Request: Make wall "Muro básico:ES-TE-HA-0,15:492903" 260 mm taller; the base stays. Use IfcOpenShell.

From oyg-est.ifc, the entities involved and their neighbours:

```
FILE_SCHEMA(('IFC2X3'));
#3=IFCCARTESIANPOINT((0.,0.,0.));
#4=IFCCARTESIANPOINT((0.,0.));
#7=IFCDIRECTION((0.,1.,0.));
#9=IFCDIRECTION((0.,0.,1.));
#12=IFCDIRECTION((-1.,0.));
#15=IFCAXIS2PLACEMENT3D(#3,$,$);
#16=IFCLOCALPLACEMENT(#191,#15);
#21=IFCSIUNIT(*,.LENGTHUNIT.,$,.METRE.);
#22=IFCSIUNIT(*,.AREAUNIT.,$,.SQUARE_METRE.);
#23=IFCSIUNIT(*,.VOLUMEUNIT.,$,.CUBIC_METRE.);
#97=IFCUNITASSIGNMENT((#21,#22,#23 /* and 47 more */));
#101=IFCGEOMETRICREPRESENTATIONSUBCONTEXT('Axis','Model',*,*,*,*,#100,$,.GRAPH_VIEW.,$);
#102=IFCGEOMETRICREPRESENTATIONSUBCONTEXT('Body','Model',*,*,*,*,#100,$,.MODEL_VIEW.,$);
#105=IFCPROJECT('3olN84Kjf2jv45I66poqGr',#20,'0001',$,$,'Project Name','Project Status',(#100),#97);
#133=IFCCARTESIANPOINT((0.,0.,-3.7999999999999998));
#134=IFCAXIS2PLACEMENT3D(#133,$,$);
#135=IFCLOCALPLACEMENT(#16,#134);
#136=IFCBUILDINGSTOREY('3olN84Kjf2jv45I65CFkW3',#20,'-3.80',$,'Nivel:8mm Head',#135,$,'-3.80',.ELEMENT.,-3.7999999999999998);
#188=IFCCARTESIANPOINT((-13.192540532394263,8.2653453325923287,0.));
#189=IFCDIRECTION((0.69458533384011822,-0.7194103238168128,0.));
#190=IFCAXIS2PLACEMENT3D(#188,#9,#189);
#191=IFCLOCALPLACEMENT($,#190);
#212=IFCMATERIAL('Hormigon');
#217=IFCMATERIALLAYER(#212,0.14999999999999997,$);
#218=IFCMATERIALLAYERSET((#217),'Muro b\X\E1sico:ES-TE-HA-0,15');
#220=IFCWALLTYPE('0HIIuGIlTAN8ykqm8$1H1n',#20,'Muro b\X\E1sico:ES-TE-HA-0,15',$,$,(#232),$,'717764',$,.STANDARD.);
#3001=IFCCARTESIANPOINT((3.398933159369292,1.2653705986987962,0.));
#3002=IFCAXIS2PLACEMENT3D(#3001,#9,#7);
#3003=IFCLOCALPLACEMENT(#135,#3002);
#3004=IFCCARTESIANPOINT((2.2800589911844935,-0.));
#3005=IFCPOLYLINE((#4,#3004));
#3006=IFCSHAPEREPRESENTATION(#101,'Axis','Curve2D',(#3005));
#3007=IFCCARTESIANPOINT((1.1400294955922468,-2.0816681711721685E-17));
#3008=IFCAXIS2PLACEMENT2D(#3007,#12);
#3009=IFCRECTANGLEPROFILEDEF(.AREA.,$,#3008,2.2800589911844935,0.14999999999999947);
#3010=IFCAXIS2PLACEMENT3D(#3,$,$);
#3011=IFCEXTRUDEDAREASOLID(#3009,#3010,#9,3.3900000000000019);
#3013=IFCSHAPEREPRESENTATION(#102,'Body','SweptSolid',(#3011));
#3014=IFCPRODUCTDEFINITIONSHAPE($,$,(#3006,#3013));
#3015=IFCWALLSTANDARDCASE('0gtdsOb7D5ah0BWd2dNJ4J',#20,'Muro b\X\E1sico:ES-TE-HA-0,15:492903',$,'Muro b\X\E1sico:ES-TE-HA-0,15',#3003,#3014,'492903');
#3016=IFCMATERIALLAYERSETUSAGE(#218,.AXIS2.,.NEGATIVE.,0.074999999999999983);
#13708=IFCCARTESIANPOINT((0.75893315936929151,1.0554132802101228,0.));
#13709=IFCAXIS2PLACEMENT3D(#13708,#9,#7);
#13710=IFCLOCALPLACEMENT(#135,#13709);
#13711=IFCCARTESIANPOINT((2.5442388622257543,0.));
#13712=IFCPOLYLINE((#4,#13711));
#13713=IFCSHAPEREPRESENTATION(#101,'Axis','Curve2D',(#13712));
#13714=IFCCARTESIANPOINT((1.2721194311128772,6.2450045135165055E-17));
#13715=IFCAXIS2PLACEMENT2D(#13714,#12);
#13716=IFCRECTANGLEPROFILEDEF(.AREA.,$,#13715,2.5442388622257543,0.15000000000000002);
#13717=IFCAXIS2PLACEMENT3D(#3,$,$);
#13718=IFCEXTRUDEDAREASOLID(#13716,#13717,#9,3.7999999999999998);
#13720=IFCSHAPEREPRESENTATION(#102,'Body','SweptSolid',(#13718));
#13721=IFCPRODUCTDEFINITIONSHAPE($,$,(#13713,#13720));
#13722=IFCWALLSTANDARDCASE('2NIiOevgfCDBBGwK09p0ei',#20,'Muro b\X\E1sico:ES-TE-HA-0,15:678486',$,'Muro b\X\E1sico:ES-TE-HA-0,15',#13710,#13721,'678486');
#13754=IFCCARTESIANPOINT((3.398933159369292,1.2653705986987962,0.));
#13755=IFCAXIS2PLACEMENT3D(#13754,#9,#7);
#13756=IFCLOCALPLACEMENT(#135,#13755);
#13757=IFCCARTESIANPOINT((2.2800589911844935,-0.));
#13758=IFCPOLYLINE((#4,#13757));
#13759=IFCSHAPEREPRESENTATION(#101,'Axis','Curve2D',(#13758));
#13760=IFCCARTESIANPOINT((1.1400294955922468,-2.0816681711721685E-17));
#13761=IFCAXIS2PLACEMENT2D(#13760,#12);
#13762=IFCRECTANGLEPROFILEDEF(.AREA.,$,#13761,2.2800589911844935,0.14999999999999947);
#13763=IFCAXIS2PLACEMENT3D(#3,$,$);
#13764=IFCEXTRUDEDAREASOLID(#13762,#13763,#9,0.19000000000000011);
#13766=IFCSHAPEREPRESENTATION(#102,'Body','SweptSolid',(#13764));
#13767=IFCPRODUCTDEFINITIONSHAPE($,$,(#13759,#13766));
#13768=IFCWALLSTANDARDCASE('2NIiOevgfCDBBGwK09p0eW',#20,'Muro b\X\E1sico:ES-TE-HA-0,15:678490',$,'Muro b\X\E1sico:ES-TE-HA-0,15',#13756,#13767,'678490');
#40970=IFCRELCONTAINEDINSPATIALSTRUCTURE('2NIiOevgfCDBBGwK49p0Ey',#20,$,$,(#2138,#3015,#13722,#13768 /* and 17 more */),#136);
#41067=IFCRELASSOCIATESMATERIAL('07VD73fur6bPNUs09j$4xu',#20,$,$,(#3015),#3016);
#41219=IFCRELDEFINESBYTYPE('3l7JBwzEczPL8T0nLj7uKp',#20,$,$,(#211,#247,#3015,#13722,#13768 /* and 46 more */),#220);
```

```python
import ifcopenshell
import ifcopenshell.geom
import ifcopenshell.util.representation
import ifcopenshell.util.shape

model = ifcopenshell.open("oyg-est.ifc")
settings = ifcopenshell.geom.settings()


def volume(element):
    """Net volume in cubic metres, openings subtracted."""
    shape = ifcopenshell.geom.create_shape(settings, element)
    return ifcopenshell.util.shape.get_volume(shape.geometry)


wall = model.by_guid("0gtdsOb7D5ah0BWd2dNJ4J")
before = volume(wall)

body = ifcopenshell.util.representation.get_representation(wall, "Model", "Body")
solid = body.Items[0]
old_height = solid.Depth
solid.Depth += 0.26
after = volume(wall)

print(f"height {old_height:g} -> {solid.Depth:g}, volume {before:.3f} -> {after:.3f} m3")

model.write("oyg-est-out.ifc")
```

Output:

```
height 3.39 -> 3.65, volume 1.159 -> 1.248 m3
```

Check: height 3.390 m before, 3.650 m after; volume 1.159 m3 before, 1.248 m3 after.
